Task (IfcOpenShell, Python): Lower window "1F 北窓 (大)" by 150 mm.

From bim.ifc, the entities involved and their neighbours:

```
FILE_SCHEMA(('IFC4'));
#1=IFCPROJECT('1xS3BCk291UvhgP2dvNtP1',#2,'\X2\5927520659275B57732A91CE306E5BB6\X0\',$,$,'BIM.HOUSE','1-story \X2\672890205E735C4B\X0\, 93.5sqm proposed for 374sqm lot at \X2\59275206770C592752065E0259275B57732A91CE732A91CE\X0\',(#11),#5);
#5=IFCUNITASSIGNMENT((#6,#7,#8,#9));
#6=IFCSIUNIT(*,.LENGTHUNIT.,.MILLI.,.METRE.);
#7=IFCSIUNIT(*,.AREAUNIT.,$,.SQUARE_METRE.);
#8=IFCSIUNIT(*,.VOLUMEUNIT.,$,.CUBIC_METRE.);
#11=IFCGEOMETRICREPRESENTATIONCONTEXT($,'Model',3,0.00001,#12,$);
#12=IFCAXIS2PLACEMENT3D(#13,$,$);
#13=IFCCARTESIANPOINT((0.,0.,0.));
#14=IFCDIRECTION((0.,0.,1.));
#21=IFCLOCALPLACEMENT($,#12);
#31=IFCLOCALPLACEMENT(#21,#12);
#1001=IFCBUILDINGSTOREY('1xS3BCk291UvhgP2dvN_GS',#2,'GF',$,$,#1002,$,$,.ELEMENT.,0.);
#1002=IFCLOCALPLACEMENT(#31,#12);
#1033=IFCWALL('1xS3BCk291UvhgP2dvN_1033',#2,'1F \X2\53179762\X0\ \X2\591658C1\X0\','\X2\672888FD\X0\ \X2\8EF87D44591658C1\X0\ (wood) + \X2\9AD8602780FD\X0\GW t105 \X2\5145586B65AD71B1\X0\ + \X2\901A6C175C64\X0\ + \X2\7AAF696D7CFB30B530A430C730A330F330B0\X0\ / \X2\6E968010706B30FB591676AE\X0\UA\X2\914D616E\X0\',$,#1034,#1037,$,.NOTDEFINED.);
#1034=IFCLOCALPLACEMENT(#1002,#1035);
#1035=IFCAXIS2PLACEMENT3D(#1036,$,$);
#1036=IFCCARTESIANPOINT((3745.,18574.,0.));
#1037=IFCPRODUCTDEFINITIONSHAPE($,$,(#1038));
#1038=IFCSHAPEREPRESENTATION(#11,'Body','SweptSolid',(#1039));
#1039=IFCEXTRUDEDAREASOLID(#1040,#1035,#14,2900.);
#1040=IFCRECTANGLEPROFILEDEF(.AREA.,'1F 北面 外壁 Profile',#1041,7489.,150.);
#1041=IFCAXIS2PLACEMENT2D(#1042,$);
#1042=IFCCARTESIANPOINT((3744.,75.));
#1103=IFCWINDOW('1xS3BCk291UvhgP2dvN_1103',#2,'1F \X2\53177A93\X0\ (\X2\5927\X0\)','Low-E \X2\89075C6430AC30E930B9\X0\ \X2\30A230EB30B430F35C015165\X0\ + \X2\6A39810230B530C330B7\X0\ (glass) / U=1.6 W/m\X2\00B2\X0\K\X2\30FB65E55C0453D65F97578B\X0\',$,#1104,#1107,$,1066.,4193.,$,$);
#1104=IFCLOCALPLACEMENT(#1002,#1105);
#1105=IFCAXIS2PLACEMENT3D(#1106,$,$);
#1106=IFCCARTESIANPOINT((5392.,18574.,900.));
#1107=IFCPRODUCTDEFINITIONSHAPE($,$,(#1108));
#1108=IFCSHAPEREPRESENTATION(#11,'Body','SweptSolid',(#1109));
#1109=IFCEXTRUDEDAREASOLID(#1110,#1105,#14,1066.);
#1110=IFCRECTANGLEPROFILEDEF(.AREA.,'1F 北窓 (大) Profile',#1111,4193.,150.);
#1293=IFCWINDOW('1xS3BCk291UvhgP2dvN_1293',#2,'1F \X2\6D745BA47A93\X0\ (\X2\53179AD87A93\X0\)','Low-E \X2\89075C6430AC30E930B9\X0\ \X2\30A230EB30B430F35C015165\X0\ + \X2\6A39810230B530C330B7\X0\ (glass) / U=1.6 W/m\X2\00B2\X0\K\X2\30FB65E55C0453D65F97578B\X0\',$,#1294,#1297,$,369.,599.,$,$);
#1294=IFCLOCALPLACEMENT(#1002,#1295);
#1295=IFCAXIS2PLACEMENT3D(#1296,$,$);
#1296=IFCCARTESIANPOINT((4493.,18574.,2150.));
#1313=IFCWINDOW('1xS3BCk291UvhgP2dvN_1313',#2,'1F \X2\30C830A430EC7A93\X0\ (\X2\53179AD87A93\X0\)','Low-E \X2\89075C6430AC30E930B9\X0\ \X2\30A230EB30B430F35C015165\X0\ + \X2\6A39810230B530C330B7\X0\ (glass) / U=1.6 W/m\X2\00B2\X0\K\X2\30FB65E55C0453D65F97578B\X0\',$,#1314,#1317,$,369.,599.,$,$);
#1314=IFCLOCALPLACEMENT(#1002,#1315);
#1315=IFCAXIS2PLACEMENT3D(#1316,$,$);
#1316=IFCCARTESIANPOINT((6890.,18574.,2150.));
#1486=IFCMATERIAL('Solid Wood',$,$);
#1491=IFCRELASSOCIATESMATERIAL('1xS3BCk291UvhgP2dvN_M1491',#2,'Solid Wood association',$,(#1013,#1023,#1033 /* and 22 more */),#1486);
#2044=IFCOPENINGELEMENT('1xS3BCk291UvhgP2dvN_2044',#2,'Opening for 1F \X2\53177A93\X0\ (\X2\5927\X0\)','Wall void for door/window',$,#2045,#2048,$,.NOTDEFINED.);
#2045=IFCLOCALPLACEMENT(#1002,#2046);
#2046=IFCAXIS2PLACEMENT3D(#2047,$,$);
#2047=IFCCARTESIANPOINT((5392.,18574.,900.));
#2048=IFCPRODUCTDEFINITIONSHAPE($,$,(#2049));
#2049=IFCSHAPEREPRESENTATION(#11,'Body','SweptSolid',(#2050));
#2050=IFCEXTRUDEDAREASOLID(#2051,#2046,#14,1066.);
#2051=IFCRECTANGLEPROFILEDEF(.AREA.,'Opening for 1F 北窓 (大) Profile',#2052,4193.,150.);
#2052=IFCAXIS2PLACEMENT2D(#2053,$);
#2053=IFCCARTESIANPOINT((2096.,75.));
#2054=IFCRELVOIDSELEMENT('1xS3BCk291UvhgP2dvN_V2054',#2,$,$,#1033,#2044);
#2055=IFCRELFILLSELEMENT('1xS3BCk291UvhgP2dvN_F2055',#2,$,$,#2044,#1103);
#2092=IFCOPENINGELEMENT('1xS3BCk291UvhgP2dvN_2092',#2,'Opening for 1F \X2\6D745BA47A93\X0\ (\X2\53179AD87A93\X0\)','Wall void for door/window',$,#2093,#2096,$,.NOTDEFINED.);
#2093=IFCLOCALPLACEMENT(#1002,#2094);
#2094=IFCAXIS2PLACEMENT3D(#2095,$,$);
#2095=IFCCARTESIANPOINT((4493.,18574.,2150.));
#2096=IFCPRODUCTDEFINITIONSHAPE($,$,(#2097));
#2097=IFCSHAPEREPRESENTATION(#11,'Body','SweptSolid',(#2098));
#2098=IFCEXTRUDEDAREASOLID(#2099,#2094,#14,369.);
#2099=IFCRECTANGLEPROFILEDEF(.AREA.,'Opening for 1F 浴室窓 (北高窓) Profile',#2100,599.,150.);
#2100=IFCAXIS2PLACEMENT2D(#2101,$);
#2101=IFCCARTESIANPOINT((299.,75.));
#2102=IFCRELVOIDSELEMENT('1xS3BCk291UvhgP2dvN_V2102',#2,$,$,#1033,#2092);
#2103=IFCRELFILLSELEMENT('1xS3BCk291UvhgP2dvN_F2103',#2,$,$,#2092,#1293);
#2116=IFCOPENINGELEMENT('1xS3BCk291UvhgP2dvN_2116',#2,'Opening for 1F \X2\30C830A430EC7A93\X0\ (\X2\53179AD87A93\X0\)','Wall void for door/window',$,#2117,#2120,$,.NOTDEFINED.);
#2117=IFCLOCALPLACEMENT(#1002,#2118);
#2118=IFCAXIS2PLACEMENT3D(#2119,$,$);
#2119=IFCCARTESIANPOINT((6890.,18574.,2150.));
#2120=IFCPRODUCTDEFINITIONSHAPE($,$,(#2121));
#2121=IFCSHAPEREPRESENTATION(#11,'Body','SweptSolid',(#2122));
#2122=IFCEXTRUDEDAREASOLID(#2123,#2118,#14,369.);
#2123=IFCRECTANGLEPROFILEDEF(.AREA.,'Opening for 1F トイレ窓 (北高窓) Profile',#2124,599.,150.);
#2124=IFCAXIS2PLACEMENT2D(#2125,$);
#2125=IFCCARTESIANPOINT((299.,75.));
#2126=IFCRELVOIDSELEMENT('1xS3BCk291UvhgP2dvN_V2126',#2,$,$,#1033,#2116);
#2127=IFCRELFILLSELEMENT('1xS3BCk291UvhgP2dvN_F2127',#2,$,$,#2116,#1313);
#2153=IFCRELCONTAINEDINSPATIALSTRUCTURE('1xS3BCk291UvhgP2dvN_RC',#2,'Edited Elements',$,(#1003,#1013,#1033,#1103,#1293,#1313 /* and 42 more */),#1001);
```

```python
import numpy as np
import ifcopenshell
import ifcopenshell.api.geometry
import ifcopenshell.util.placement
import ifcopenshell.util.unit

model = ifcopenshell.open("bim.ifc")
unit_scale = ifcopenshell.util.unit.calculate_unit_scale(model)

window = model.by_guid("1xS3BCk291UvhgP2dvN_1103")
opening = window.FillsVoids[0].RelatingOpeningElement
dz = -0.15 / unit_scale

shift = np.array([0.0, 0.0, dz])
# The window is not placed relative to its opening, so move both.
for product in (opening, window):
    matrix = ifcopenshell.util.placement.get_local_placement(product.ObjectPlacement)
    matrix[:3, 3] += shift
    ifcopenshell.api.geometry.edit_object_placement(model, product=product, matrix=matrix, is_si=False)

print(f"moved by {dz * unit_scale:+.3f} m")

model.write("bim-out.ifc")
```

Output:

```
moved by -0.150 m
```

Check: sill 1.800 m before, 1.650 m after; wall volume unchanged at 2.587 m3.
